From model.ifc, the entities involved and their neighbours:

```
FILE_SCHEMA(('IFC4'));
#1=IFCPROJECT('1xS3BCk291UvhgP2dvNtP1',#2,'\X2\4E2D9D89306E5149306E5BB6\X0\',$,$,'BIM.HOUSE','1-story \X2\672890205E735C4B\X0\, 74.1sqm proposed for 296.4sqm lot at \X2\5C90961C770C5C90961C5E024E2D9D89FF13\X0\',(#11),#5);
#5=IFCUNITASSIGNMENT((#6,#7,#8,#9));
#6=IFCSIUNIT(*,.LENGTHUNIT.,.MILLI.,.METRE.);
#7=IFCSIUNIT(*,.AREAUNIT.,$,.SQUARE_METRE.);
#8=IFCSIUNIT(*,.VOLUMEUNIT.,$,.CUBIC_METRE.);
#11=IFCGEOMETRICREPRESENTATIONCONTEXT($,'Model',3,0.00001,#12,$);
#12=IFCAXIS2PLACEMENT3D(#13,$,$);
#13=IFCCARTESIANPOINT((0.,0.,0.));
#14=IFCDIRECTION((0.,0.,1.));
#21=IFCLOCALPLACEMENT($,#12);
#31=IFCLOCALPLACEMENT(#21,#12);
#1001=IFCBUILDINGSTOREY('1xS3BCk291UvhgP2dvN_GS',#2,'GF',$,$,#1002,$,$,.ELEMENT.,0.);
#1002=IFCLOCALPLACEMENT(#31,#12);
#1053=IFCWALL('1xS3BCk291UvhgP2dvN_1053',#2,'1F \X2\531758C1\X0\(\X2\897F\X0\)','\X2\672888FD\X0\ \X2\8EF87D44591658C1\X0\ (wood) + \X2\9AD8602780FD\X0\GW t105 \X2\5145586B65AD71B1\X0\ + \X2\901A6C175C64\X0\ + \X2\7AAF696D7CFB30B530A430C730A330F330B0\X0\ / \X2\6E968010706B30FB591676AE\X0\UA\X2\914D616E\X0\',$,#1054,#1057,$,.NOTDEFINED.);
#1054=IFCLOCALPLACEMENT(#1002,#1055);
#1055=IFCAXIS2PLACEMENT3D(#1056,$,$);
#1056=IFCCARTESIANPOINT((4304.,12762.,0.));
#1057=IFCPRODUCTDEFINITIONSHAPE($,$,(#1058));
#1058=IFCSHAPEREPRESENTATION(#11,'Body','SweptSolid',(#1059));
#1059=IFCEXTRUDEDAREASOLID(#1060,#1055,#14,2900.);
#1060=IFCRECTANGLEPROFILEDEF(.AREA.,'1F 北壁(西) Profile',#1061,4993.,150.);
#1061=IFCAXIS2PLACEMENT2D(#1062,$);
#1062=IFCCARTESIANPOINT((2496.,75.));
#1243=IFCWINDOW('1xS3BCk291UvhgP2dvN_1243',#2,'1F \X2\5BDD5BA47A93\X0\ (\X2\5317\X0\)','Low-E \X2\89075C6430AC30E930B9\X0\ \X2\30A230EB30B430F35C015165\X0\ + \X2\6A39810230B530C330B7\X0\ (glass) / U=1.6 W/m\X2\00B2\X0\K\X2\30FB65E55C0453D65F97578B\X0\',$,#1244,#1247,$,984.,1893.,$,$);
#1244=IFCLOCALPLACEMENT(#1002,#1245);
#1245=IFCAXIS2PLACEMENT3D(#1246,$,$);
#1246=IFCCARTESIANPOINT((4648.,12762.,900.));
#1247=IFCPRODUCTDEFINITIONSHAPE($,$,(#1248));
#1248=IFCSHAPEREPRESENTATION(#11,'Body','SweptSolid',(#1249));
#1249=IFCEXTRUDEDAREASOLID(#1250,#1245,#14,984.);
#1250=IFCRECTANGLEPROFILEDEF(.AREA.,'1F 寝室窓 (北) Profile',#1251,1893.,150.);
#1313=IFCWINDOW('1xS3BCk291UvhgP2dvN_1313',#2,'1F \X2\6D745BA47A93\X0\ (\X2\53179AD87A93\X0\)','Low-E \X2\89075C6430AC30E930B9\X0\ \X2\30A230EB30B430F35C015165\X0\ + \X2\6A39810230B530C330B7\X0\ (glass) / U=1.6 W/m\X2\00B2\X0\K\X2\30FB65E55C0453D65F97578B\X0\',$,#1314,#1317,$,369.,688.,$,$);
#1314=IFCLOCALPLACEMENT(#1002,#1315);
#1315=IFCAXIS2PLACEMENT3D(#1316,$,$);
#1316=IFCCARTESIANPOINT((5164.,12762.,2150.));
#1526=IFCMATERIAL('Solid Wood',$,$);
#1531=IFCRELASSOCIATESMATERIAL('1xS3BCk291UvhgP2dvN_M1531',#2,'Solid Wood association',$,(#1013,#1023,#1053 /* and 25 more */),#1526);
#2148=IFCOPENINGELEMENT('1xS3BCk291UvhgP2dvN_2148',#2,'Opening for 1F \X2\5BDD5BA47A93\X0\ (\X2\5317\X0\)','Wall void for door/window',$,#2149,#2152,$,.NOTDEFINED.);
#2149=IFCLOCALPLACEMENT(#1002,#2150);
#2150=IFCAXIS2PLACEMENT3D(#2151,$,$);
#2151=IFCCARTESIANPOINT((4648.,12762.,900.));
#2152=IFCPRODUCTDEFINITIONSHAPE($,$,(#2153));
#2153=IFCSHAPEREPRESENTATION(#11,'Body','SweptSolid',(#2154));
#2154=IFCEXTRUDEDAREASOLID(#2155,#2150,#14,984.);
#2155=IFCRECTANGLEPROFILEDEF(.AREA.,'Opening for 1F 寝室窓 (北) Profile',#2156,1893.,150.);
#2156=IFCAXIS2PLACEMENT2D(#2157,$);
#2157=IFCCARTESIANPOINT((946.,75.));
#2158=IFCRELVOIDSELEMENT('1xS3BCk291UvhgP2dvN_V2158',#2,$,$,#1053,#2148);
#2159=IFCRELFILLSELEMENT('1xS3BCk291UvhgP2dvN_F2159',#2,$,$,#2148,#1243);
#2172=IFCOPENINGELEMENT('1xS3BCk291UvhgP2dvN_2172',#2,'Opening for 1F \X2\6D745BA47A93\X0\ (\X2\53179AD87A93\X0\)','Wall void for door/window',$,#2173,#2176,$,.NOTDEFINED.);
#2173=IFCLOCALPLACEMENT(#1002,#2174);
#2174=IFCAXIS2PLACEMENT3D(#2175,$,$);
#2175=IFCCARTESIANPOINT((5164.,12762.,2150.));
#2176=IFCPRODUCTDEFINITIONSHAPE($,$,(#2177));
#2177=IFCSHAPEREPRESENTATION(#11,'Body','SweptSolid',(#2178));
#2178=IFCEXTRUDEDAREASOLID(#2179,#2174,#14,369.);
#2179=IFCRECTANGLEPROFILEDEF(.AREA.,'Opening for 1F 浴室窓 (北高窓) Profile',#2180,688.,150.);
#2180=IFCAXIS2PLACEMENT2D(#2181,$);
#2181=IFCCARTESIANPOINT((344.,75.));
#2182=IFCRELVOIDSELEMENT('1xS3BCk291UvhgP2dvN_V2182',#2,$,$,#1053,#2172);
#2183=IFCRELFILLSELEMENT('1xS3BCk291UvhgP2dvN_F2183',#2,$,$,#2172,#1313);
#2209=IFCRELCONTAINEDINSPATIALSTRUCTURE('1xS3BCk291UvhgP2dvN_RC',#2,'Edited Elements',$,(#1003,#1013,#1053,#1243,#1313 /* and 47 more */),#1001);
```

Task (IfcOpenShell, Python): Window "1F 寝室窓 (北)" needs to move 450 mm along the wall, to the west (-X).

```python
import ifcopenshell
import ifcopenshell.api.geometry
import ifcopenshell.util.placement

model = ifcopenshell.open("model.ifc")

window = model.by_guid("1xS3BCk291UvhgP2dvN_1243")
opening = window.FillsVoids[0].RelatingOpeningElement
wall = opening.VoidsElements[0].RelatingBuildingElement

wall_matrix = ifcopenshell.util.placement.get_local_placement(wall.ObjectPlacement)
shift = wall_matrix[:3, 0] * -450.0
before = ifcopenshell.util.placement.get_local_placement(window.ObjectPlacement)[:3, 3].copy()

# The window is not placed relative to its opening, so move both.
for product in (opening, window):
    matrix = ifcopenshell.util.placement.get_local_placement(product.ObjectPlacement)
    matrix[:3, 3] += shift
    ifcopenshell.api.geometry.edit_object_placement(model, product=product, matrix=matrix, is_si=False)

after = ifcopenshell.util.placement.get_local_placement(window.ObjectPlacement)[:3, 3]
print("window moved by", (after - before).round(3) + 0.0)

model.write("model_edited.ifc")
```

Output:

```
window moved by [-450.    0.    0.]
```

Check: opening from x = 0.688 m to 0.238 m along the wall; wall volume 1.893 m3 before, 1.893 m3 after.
